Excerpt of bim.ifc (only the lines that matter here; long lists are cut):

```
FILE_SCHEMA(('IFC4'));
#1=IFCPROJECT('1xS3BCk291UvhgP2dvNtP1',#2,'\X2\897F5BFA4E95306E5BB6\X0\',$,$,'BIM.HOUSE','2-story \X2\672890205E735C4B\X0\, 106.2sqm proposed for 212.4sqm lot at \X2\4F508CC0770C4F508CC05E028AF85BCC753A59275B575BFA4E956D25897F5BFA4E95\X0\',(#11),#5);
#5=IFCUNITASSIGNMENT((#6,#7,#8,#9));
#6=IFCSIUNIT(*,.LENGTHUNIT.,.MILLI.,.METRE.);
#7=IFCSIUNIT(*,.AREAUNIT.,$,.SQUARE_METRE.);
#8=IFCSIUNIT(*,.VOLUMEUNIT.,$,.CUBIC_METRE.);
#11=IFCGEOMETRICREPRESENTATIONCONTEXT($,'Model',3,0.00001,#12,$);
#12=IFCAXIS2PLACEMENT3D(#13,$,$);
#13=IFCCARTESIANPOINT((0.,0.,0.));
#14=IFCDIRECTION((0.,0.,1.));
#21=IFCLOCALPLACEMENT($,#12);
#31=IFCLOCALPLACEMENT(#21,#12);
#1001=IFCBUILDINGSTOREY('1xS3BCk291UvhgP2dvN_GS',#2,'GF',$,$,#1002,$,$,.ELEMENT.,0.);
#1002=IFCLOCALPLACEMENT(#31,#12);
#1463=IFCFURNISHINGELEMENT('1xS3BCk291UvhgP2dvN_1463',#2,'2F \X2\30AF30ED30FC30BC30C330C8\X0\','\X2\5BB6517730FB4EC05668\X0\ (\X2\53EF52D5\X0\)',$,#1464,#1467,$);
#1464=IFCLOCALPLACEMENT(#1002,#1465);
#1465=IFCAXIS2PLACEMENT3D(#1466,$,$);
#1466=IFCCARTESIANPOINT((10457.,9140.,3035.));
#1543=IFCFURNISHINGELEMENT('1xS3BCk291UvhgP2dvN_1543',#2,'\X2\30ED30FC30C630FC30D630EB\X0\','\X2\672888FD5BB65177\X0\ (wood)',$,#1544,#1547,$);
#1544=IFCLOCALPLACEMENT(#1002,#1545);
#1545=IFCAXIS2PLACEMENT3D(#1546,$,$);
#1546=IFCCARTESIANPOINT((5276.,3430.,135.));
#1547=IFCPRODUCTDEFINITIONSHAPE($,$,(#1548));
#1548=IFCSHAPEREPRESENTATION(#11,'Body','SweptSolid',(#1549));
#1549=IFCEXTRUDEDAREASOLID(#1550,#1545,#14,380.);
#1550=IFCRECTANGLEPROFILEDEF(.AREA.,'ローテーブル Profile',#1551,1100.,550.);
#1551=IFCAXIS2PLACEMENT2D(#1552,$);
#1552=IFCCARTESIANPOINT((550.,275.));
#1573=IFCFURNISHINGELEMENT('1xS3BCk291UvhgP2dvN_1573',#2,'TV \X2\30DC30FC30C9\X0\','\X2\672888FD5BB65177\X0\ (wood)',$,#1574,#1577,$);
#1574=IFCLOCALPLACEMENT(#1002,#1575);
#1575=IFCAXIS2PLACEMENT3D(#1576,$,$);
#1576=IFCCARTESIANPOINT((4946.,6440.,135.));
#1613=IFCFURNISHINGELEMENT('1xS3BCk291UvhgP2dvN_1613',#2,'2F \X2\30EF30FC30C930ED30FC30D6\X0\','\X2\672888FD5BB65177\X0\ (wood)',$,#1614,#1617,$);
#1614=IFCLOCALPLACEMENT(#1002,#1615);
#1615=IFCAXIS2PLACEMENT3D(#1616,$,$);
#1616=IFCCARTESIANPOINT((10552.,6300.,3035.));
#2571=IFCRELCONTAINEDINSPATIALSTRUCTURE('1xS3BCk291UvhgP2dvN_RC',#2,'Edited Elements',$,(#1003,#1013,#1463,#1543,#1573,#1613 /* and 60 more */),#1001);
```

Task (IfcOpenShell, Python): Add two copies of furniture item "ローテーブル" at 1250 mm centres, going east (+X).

```python
import numpy as np
import ifcopenshell
import ifcopenshell.api.geometry
import ifcopenshell.api.root
import ifcopenshell.util.element
import ifcopenshell.util.placement
import ifcopenshell.util.unit

model = ifcopenshell.open("bim.ifc")
unit_scale = ifcopenshell.util.unit.calculate_unit_scale(model)


def reuse_history(source, copy):
    """copy_class also copies each property set's owner history, people and application; keep the originals."""
    for rel in copy.IsDefinedBy:
        if rel.is_a("IfcRelDefinesByProperties") and (history := rel.RelatingPropertyDefinition.OwnerHistory):
            rel.RelatingPropertyDefinition.OwnerHistory = source.OwnerHistory
            ifcopenshell.util.element.remove_deep2(model, history)


source = model.by_guid("1xS3BCk291UvhgP2dvN_1543")
base = ifcopenshell.util.placement.get_local_placement(source.ObjectPlacement)
step = np.array([1.0, 0.0, 0.0]) * 1.25 / unit_scale

for i in range(1, 3):
    copy = ifcopenshell.api.root.copy_class(model, product=source)
    copy.Representation = ifcopenshell.util.element.copy_deep(
        model, source.Representation, exclude=["IfcGeometricRepresentationContext", "IfcRepresentationMap"]
    )
    reuse_history(source, copy)
    matrix = base.copy()
    matrix[:3, 3] += i * step
    print("added at", matrix[:3, 3].round(3) + 0.0)
    ifcopenshell.api.geometry.edit_object_placement(model, product=copy, matrix=matrix, is_si=False)

model.write("bim-out.ifc")
```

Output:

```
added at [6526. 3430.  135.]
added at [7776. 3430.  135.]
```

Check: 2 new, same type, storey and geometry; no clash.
